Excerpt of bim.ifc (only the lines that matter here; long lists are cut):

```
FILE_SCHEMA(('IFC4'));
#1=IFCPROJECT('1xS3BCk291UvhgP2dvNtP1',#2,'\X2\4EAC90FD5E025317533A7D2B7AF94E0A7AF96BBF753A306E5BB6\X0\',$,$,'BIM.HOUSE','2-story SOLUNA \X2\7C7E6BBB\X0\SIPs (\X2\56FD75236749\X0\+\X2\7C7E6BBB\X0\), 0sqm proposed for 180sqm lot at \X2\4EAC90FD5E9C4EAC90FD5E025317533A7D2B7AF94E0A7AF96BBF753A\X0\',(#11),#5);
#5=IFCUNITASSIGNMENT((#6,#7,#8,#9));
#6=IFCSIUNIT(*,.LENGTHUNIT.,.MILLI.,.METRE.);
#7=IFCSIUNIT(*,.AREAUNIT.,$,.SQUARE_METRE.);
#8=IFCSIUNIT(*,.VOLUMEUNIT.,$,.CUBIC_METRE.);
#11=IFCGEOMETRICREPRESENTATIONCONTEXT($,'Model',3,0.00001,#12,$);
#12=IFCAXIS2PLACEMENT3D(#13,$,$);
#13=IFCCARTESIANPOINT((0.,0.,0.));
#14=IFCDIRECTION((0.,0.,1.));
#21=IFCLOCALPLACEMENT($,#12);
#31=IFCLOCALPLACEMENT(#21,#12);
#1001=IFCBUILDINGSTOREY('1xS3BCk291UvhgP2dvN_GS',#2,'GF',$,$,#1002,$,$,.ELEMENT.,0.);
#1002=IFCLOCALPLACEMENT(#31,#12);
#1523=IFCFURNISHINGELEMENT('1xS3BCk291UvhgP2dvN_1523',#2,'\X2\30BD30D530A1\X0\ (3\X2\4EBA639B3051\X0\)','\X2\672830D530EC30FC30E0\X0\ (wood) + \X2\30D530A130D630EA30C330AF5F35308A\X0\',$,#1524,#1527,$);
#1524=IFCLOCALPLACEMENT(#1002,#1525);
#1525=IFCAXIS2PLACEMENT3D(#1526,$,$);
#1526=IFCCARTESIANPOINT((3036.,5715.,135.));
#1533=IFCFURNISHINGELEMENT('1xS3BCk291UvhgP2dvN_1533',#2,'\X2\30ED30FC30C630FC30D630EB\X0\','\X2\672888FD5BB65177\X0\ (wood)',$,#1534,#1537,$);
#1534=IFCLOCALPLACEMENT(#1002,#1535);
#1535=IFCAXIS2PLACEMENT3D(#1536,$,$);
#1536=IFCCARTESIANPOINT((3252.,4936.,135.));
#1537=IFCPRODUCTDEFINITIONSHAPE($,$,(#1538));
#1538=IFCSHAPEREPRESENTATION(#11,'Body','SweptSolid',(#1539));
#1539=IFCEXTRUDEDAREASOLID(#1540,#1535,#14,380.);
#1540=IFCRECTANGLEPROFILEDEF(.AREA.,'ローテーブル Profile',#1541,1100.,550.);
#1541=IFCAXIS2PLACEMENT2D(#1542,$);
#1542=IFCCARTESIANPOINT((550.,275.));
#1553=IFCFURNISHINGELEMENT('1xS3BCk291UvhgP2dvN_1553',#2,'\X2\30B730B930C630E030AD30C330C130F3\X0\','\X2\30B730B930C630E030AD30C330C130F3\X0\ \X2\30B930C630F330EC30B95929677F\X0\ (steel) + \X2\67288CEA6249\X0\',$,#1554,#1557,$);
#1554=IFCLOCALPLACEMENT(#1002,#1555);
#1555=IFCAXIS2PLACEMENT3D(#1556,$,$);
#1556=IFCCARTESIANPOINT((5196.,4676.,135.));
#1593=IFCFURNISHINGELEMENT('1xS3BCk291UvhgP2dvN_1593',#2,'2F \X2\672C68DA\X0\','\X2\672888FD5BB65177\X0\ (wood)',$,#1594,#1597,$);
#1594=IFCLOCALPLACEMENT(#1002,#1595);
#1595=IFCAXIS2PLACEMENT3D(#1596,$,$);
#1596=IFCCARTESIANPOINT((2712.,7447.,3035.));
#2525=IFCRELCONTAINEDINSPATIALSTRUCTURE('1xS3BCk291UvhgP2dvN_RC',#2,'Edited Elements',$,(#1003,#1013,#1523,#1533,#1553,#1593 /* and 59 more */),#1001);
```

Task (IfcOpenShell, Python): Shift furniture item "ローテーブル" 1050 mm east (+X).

```python
import ifcopenshell
import ifcopenshell.api.geometry
import ifcopenshell.util.placement
import ifcopenshell.util.unit

model = ifcopenshell.open("bim.ifc")
unit_scale = ifcopenshell.util.unit.calculate_unit_scale(model)

item = model.by_guid("1xS3BCk291UvhgP2dvN_1533")
matrix = ifcopenshell.util.placement.get_local_placement(item.ObjectPlacement)
matrix[0, 3] += 1.05 / unit_scale
ifcopenshell.api.geometry.edit_object_placement(model, product=item, matrix=matrix, is_si=False)

print(ifcopenshell.util.placement.get_local_placement(item.ObjectPlacement).round(3) + 0.0)

model.write("bim_edited.ifc")
```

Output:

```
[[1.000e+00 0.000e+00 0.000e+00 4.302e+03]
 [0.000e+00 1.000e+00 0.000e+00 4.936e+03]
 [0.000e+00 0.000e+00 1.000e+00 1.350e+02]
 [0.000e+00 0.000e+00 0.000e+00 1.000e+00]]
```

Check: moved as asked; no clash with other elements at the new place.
